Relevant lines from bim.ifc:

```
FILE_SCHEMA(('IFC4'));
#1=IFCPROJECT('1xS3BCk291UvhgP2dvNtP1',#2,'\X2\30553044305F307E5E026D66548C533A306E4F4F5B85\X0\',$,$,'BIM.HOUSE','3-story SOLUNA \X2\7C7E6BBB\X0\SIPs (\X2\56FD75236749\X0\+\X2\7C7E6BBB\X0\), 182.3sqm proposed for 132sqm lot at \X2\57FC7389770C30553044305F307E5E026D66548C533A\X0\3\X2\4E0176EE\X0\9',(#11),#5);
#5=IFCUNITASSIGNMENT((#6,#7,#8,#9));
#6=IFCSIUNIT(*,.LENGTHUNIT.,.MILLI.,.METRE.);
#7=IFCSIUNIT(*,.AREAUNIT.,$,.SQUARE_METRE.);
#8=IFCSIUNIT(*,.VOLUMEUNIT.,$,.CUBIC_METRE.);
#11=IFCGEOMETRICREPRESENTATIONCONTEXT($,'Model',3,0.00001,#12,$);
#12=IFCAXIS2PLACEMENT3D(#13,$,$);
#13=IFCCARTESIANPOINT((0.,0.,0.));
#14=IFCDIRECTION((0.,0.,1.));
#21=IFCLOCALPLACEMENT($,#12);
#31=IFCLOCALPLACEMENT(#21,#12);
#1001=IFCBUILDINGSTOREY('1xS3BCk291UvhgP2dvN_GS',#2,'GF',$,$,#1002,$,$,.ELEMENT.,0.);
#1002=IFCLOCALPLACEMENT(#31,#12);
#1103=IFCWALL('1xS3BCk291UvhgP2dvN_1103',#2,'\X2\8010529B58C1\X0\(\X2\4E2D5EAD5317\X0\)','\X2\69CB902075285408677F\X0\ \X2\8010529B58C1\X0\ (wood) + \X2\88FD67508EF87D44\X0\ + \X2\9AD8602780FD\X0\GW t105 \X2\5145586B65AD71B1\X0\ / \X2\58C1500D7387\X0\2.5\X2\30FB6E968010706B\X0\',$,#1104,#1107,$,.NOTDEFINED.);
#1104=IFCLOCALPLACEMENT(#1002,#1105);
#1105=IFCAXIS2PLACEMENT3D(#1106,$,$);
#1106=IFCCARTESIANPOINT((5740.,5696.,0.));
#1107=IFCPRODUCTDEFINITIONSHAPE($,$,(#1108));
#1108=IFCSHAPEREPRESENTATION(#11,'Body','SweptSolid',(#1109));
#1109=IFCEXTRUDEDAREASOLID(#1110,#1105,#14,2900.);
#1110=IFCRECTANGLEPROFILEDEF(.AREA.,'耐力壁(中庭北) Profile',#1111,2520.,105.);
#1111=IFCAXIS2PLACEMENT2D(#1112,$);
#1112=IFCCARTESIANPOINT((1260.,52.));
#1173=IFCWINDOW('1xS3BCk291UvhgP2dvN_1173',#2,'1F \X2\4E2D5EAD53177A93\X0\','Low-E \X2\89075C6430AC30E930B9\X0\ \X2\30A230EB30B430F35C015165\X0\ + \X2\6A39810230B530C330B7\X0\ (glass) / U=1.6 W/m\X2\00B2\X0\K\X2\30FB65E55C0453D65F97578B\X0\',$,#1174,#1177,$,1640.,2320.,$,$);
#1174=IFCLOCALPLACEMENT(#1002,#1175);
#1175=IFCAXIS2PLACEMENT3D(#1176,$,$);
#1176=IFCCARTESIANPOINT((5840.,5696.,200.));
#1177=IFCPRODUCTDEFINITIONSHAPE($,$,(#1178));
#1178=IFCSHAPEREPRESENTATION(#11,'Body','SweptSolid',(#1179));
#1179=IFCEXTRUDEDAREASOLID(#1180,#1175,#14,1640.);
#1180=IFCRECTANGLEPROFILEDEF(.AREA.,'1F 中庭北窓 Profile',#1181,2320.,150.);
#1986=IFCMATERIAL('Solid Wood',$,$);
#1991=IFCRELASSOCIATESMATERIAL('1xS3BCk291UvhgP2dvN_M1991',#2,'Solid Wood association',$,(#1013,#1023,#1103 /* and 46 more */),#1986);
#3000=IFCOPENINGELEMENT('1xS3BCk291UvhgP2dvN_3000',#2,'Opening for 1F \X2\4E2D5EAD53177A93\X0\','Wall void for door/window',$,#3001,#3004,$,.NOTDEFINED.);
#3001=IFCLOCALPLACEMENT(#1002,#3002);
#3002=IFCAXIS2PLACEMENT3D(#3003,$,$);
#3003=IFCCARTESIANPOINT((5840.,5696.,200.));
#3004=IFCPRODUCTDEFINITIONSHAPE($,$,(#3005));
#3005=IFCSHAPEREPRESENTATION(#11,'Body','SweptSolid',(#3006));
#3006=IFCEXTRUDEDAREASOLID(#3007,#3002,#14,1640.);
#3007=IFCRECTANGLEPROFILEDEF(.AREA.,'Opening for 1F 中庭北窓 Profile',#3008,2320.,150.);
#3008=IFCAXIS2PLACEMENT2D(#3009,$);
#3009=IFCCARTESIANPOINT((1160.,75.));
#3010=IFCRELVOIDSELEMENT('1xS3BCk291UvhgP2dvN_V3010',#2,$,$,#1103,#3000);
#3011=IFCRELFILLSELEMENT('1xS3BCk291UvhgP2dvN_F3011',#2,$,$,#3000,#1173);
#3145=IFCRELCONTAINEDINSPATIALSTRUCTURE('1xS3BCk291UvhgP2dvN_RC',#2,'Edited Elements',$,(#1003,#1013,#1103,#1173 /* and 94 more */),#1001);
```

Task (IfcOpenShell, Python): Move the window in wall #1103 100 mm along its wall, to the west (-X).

```python
import ifcopenshell
import ifcopenshell.api.geometry
import ifcopenshell.util.placement

model = ifcopenshell.open("bim.ifc")

window = model.by_id(1173)
opening = window.FillsVoids[0].RelatingOpeningElement
wall = opening.VoidsElements[0].RelatingBuildingElement

wall_matrix = ifcopenshell.util.placement.get_local_placement(wall.ObjectPlacement)
shift = wall_matrix[:3, 0] * -100.0
before = ifcopenshell.util.placement.get_local_placement(window.ObjectPlacement)[:3, 3].copy()

# The window is not placed relative to its opening, so move both.
for product in (opening, window):
    matrix = ifcopenshell.util.placement.get_local_placement(product.ObjectPlacement)
    matrix[:3, 3] += shift
    ifcopenshell.api.geometry.edit_object_placement(model, product=product, matrix=matrix, is_si=False)

after = ifcopenshell.util.placement.get_local_placement(window.ObjectPlacement)[:3, 3]
print("window moved by", (after - before).round(3) + 0.0)

model.write("bim_updated.ifc")
```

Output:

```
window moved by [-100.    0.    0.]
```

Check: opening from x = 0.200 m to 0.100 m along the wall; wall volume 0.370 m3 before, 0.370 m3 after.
